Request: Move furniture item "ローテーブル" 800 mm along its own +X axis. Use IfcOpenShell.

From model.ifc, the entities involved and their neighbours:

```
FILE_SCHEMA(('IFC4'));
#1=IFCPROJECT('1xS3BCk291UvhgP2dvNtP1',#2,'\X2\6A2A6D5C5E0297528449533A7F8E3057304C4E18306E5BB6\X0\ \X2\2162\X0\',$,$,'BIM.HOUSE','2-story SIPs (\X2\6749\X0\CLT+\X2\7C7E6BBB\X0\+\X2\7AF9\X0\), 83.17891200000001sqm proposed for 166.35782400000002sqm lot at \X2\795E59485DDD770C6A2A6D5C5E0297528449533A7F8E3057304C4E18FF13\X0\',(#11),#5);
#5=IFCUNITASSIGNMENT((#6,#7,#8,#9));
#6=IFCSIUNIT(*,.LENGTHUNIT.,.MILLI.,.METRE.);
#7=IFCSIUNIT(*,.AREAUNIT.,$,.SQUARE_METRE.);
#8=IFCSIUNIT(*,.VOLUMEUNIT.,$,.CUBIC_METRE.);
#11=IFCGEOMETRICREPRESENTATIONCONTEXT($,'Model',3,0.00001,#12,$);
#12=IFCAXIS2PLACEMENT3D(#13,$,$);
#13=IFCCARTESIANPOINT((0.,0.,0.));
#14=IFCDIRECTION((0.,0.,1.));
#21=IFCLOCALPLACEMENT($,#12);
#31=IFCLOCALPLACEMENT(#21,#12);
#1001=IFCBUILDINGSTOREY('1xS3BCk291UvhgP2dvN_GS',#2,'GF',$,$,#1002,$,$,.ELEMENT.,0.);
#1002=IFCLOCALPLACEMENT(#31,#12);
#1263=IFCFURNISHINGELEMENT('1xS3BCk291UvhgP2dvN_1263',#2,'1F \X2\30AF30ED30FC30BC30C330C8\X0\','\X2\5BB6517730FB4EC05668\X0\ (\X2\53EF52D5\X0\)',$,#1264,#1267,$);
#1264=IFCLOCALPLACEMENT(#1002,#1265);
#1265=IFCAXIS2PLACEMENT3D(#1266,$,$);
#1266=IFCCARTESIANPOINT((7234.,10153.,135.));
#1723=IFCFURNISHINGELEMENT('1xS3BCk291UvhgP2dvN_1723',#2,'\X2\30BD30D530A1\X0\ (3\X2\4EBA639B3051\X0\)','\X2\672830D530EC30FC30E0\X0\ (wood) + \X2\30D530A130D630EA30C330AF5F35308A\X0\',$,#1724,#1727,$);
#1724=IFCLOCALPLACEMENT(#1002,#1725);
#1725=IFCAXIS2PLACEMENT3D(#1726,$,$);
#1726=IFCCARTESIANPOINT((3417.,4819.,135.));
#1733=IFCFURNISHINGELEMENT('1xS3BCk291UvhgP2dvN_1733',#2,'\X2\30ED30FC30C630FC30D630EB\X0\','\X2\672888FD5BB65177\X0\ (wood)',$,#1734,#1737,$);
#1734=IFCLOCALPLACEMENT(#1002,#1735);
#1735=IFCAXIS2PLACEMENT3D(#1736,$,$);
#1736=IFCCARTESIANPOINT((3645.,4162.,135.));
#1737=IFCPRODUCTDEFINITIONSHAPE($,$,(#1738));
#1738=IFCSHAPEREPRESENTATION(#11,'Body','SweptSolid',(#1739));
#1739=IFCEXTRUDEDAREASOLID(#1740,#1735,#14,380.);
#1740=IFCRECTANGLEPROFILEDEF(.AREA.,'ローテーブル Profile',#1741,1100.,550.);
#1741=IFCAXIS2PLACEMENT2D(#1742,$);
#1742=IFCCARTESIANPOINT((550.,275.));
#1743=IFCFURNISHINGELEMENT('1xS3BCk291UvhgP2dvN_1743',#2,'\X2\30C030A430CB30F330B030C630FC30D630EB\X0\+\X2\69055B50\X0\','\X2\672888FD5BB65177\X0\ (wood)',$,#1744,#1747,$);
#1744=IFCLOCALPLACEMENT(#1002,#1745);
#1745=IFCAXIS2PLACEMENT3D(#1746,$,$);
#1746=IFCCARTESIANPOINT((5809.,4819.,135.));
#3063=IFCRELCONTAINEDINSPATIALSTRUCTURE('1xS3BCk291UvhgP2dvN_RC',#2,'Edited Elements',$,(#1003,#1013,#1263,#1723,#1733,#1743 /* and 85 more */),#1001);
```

```python
import ifcopenshell
import ifcopenshell.api.geometry
import ifcopenshell.util.placement
import ifcopenshell.util.unit

model = ifcopenshell.open("model.ifc")
unit_scale = ifcopenshell.util.unit.calculate_unit_scale(model)

item = model.by_guid("1xS3BCk291UvhgP2dvN_1733")
matrix = ifcopenshell.util.placement.get_local_placement(item.ObjectPlacement)
matrix[:3, 3] += matrix[:3, 0] * 0.8 / unit_scale
ifcopenshell.api.geometry.edit_object_placement(model, product=item, matrix=matrix, is_si=False)

print(ifcopenshell.util.placement.get_local_placement(item.ObjectPlacement).round(3) + 0.0)

model.write("model_updated.ifc")
```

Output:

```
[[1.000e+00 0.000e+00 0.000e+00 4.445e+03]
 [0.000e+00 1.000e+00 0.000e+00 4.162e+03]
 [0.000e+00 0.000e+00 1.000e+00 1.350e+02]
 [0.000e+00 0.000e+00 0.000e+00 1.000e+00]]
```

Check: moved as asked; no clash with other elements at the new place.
